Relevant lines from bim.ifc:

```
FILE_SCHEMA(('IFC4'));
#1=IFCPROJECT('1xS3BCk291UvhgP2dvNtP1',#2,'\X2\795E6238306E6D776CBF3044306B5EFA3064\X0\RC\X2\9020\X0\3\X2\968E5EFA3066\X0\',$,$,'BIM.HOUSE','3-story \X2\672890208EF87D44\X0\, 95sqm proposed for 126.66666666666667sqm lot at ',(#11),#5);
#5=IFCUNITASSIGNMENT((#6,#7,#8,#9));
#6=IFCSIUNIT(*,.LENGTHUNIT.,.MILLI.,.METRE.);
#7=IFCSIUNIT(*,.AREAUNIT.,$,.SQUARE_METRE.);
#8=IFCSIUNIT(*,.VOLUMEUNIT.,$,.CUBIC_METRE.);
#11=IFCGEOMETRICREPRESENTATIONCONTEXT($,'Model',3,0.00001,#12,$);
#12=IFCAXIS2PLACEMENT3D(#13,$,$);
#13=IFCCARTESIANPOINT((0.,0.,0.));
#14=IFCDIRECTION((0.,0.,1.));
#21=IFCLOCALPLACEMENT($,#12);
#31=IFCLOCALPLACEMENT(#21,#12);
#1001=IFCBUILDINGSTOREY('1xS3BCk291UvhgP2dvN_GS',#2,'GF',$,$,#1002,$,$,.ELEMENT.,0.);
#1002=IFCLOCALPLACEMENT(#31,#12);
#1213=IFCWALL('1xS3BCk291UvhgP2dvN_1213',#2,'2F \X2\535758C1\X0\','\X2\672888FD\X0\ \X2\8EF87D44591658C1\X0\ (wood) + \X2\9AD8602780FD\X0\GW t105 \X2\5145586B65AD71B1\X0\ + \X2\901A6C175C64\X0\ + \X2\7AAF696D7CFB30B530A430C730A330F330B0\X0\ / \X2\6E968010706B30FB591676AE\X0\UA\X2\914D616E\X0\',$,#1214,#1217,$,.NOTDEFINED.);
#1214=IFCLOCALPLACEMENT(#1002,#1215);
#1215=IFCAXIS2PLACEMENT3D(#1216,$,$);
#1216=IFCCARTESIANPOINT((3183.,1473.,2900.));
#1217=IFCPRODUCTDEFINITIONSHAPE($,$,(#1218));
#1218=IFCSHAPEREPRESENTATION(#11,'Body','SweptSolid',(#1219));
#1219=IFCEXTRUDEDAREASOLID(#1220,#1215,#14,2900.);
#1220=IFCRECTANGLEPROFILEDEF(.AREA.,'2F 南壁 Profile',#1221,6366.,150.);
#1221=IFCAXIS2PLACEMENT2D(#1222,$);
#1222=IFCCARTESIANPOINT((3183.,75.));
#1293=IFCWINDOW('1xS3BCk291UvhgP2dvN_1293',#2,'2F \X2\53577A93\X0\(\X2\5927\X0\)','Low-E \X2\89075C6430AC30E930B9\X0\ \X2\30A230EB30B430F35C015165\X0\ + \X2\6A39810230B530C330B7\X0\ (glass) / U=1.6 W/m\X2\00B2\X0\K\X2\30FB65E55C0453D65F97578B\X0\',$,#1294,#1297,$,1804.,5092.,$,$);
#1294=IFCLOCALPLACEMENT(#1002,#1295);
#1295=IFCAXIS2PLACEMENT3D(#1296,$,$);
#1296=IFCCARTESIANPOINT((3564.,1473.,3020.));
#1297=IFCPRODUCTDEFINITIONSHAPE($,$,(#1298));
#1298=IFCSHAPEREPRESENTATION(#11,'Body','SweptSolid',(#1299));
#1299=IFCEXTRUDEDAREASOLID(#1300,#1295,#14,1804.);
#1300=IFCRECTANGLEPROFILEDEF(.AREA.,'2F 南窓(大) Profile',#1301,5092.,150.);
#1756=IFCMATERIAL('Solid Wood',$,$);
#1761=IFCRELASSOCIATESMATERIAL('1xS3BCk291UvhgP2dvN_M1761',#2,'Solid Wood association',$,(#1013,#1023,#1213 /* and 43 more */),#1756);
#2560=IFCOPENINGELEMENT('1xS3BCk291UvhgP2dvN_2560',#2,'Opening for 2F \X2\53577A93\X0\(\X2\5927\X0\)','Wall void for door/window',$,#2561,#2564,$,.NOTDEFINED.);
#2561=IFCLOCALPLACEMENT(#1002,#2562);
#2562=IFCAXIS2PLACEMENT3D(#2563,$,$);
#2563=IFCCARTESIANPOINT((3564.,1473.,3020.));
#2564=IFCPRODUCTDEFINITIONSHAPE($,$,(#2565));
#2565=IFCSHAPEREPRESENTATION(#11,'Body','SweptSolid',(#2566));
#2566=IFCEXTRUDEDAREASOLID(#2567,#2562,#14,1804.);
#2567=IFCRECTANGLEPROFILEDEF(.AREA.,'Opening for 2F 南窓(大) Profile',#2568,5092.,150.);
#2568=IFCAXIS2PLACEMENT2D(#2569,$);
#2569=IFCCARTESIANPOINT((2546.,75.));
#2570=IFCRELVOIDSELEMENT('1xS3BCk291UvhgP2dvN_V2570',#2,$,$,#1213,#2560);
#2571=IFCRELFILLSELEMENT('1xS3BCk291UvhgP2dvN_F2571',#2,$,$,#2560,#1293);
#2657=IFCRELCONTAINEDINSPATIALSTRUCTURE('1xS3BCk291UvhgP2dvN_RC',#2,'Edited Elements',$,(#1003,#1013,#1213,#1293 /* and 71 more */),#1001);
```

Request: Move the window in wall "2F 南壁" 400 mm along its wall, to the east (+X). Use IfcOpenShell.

```python
import ifcopenshell
import ifcopenshell.api.geometry
import ifcopenshell.util.placement
import ifcopenshell.util.unit

model = ifcopenshell.open("bim.ifc")
unit_scale = ifcopenshell.util.unit.calculate_unit_scale(model)

window = model.by_guid("1xS3BCk291UvhgP2dvN_1293")
opening = window.FillsVoids[0].RelatingOpeningElement
wall = opening.VoidsElements[0].RelatingBuildingElement

wall_matrix = ifcopenshell.util.placement.get_local_placement(wall.ObjectPlacement)
shift = wall_matrix[:3, 0] * 0.4 / unit_scale
before = ifcopenshell.util.placement.get_local_placement(window.ObjectPlacement)[:3, 3].copy()

# The window is not placed relative to its opening, so move both.
for product in (opening, window):
    matrix = ifcopenshell.util.placement.get_local_placement(product.ObjectPlacement)
    matrix[:3, 3] += shift
    ifcopenshell.api.geometry.edit_object_placement(model, product=product, matrix=matrix, is_si=False)

after = ifcopenshell.util.placement.get_local_placement(window.ObjectPlacement)[:3, 3]
print("window moved by", (after - before).round(3) + 0.0)

model.write("bim-out.ifc")
```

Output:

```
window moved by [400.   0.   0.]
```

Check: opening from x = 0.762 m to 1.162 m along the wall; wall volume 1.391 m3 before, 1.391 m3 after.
